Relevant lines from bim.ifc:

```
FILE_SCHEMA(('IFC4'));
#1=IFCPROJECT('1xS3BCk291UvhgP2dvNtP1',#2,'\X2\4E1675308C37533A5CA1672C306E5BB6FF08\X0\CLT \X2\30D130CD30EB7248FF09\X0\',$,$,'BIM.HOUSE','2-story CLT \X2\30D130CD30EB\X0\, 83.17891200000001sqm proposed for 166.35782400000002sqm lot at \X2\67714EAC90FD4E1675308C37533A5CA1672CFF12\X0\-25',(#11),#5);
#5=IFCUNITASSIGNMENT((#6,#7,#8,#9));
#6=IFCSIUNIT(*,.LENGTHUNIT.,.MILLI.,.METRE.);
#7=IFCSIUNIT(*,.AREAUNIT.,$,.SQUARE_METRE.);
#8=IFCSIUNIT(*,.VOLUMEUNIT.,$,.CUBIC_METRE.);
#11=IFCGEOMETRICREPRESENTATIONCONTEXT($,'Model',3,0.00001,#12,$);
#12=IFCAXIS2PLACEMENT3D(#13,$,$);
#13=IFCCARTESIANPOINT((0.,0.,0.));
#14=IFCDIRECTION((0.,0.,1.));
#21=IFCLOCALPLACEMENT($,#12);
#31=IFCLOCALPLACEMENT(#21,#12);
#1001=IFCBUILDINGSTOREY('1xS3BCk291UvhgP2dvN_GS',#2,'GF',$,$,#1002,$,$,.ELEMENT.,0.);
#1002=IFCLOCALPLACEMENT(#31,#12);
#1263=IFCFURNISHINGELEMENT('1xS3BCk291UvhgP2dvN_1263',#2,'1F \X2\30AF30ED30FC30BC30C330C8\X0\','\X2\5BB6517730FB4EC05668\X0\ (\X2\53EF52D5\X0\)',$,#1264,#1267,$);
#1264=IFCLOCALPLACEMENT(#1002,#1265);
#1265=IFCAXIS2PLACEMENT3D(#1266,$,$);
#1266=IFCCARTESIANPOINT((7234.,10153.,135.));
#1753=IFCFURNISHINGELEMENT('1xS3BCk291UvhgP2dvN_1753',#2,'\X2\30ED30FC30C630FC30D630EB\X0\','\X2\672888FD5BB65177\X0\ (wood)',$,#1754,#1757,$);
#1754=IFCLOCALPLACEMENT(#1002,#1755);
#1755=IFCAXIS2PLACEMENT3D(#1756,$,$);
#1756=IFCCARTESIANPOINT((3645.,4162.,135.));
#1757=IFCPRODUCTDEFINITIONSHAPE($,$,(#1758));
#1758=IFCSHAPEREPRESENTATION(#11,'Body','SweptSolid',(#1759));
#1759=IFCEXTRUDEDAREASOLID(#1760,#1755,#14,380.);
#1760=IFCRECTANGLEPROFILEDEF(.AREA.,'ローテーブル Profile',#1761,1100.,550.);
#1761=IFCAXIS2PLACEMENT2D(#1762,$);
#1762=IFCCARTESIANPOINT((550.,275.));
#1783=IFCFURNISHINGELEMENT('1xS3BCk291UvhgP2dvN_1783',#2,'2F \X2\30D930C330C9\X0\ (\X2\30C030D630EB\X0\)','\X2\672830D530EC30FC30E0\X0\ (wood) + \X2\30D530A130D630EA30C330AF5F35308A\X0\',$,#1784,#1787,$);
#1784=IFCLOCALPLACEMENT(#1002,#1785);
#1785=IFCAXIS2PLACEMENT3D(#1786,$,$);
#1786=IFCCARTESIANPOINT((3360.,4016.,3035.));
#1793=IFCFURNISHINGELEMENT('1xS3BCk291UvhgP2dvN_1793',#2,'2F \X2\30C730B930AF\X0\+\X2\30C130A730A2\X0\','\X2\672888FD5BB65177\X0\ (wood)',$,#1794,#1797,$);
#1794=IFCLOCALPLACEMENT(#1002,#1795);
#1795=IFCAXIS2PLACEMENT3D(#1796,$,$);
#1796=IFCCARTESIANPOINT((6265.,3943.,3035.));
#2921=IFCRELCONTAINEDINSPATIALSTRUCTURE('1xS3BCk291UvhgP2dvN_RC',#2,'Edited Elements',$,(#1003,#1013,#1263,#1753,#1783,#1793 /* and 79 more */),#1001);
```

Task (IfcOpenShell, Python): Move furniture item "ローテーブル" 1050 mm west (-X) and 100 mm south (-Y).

```python
import ifcopenshell
import ifcopenshell.api.geometry
import ifcopenshell.util.placement

model = ifcopenshell.open("bim.ifc")

item = model.by_guid("1xS3BCk291UvhgP2dvN_1753")
matrix = ifcopenshell.util.placement.get_local_placement(item.ObjectPlacement)
matrix[0, 3] -= 1050.0
matrix[1, 3] -= 100.0
ifcopenshell.api.geometry.edit_object_placement(model, product=item, matrix=matrix, is_si=False)

print(ifcopenshell.util.placement.get_local_placement(item.ObjectPlacement).round(3) + 0.0)

model.write("bim_v2.ifc")
```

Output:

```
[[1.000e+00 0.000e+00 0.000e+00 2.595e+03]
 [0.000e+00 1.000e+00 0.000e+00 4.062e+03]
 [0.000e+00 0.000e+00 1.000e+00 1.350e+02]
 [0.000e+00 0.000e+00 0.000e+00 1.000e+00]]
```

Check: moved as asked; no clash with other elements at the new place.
